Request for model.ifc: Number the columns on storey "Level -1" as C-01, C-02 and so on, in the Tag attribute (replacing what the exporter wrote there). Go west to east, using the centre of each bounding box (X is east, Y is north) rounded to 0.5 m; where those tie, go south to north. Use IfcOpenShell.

First a look at what the model holds.

```python
import ifcopenshell
import ifcopenshell.util.element
import ifcopenshell.util.placement

model = ifcopenshell.open("model.ifc")
print(model.schema)
storey = next(s for s in model.by_type("IfcBuildingStorey") if s.Name == "Level -1")
columns = [e for e in ifcopenshell.util.element.get_decomposition(storey) if e.is_a("IfcColumn")]
for e in sorted(columns, key=lambda e: e.id()):
    origin = ifcopenshell.util.placement.get_local_placement(e.ObjectPlacement)[:3, 3]
    print(e.id(), e.Tag, e.Name, origin.round(2) + 0.0, sep=" | ")
```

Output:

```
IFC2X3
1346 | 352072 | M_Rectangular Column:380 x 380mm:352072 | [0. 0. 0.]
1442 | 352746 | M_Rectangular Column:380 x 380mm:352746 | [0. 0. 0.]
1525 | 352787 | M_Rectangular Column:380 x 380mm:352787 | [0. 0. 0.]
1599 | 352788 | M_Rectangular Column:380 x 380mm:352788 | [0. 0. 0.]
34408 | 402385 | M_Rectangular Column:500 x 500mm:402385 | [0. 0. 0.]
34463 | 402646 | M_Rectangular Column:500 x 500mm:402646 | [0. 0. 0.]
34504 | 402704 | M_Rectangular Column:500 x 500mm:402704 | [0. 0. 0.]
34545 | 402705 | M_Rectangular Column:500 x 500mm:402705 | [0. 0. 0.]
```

```python
import ifcopenshell
import ifcopenshell.geom
import ifcopenshell.util.element
import ifcopenshell.util.shape

model = ifcopenshell.open("model.ifc")
settings = ifcopenshell.geom.settings()
settings.set("use-world-coords", True)


def centre(element):
    shape = ifcopenshell.geom.create_shape(settings, element)
    return ifcopenshell.util.shape.get_bbox_centroid(shape.geometry)


storey = next(s for s in model.by_type("IfcBuildingStorey") if s.Name == "Level -1")
columns = [e for e in ifcopenshell.util.element.get_decomposition(storey) if e.is_a("IfcColumn")]

# Insertion points can sit at a corner or the storey origin, so sort by the geometry (in metres).
centres = {e: centre(e) for e in columns}
columns.sort(key=lambda e: (round(centres[e][0] / 0.5), centres[e][1]))

for i, e in enumerate(columns, start=1):
    number = f"C-{i:02d}"
    e.Tag = number
    print(e.id(), number)

model.write("model_rev.ifc")
```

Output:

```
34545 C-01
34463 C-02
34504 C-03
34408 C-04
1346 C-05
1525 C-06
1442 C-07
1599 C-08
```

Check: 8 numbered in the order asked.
